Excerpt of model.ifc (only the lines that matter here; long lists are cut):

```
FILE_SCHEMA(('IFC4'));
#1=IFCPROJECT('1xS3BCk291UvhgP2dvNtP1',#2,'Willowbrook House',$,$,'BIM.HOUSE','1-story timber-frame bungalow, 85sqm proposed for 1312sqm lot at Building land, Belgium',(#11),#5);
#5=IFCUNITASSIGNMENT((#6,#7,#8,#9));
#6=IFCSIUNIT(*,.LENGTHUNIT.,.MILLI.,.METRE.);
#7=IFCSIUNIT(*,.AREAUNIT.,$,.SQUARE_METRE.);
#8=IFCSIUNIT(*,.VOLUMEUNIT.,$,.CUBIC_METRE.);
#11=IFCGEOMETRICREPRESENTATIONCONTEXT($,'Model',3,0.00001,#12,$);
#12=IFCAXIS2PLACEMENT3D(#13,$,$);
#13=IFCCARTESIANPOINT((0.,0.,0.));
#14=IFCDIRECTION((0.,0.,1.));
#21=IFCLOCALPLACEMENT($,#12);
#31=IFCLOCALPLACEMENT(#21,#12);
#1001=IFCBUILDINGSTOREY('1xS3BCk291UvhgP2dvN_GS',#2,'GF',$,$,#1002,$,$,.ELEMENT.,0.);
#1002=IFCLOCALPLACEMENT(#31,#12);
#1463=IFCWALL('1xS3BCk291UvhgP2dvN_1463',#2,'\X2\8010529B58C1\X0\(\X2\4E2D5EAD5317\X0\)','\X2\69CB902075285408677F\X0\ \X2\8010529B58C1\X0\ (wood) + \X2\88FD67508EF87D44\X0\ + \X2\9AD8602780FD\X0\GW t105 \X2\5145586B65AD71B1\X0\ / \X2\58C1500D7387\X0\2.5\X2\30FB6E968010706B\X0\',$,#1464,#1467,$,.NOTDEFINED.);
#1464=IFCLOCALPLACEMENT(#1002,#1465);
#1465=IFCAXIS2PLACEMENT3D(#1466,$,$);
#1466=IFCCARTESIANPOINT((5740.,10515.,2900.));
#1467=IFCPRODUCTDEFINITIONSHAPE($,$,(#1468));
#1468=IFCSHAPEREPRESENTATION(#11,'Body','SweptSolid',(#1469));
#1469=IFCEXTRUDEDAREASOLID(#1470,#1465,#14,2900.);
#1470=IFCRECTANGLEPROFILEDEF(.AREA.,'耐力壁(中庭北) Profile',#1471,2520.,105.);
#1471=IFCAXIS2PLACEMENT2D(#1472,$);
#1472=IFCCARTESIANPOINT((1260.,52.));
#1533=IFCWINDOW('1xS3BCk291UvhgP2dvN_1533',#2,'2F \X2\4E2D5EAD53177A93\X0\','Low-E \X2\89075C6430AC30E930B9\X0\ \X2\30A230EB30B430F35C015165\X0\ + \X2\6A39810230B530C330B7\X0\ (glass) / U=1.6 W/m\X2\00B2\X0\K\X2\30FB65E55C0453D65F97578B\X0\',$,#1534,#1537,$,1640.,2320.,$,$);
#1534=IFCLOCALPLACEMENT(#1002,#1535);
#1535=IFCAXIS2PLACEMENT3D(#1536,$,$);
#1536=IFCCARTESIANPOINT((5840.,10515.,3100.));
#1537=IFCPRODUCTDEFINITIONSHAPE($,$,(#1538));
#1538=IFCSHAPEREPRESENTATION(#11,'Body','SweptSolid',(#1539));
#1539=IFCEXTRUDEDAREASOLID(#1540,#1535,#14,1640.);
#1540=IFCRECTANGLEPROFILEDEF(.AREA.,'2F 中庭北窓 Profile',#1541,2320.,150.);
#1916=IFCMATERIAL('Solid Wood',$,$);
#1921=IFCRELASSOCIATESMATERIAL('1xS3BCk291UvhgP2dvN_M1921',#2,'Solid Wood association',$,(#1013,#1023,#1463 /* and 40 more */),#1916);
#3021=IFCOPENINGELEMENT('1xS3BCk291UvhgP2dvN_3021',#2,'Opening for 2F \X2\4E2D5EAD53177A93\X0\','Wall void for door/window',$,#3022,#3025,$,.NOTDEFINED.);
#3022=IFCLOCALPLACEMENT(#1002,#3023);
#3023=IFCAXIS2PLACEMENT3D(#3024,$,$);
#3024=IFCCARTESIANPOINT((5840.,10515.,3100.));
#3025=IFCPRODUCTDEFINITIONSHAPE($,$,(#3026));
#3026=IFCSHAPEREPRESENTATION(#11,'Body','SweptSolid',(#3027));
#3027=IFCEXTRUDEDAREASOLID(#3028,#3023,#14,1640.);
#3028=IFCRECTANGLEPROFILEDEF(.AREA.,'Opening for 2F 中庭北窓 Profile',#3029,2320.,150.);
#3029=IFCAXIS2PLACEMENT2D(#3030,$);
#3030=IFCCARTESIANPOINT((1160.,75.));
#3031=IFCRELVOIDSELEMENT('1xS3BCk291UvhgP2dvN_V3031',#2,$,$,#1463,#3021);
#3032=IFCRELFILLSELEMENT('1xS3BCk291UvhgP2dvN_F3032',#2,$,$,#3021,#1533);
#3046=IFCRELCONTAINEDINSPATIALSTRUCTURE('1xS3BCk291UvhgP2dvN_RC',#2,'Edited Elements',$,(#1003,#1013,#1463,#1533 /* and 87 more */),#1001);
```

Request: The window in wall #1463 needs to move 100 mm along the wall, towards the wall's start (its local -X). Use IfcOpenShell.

```python
import ifcopenshell
import ifcopenshell.api.geometry
import ifcopenshell.util.placement

model = ifcopenshell.open("model.ifc")

window = model.by_guid("1xS3BCk291UvhgP2dvN_1533")
opening = window.FillsVoids[0].RelatingOpeningElement
wall = opening.VoidsElements[0].RelatingBuildingElement

wall_matrix = ifcopenshell.util.placement.get_local_placement(wall.ObjectPlacement)
shift = wall_matrix[:3, 0] * -100.0
before = ifcopenshell.util.placement.get_local_placement(window.ObjectPlacement)[:3, 3].copy()

# The window is not placed relative to its opening, so move both.
for product in (opening, window):
    matrix = ifcopenshell.util.placement.get_local_placement(product.ObjectPlacement)
    matrix[:3, 3] += shift
    ifcopenshell.api.geometry.edit_object_placement(model, product=product, matrix=matrix, is_si=False)

after = ifcopenshell.util.placement.get_local_placement(window.ObjectPlacement)[:3, 3]
print("window moved by", (after - before).round(3) + 0.0)

model.write("model_updated.ifc")
```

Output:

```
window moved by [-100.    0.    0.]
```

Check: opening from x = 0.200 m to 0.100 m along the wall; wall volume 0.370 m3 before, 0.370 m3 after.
